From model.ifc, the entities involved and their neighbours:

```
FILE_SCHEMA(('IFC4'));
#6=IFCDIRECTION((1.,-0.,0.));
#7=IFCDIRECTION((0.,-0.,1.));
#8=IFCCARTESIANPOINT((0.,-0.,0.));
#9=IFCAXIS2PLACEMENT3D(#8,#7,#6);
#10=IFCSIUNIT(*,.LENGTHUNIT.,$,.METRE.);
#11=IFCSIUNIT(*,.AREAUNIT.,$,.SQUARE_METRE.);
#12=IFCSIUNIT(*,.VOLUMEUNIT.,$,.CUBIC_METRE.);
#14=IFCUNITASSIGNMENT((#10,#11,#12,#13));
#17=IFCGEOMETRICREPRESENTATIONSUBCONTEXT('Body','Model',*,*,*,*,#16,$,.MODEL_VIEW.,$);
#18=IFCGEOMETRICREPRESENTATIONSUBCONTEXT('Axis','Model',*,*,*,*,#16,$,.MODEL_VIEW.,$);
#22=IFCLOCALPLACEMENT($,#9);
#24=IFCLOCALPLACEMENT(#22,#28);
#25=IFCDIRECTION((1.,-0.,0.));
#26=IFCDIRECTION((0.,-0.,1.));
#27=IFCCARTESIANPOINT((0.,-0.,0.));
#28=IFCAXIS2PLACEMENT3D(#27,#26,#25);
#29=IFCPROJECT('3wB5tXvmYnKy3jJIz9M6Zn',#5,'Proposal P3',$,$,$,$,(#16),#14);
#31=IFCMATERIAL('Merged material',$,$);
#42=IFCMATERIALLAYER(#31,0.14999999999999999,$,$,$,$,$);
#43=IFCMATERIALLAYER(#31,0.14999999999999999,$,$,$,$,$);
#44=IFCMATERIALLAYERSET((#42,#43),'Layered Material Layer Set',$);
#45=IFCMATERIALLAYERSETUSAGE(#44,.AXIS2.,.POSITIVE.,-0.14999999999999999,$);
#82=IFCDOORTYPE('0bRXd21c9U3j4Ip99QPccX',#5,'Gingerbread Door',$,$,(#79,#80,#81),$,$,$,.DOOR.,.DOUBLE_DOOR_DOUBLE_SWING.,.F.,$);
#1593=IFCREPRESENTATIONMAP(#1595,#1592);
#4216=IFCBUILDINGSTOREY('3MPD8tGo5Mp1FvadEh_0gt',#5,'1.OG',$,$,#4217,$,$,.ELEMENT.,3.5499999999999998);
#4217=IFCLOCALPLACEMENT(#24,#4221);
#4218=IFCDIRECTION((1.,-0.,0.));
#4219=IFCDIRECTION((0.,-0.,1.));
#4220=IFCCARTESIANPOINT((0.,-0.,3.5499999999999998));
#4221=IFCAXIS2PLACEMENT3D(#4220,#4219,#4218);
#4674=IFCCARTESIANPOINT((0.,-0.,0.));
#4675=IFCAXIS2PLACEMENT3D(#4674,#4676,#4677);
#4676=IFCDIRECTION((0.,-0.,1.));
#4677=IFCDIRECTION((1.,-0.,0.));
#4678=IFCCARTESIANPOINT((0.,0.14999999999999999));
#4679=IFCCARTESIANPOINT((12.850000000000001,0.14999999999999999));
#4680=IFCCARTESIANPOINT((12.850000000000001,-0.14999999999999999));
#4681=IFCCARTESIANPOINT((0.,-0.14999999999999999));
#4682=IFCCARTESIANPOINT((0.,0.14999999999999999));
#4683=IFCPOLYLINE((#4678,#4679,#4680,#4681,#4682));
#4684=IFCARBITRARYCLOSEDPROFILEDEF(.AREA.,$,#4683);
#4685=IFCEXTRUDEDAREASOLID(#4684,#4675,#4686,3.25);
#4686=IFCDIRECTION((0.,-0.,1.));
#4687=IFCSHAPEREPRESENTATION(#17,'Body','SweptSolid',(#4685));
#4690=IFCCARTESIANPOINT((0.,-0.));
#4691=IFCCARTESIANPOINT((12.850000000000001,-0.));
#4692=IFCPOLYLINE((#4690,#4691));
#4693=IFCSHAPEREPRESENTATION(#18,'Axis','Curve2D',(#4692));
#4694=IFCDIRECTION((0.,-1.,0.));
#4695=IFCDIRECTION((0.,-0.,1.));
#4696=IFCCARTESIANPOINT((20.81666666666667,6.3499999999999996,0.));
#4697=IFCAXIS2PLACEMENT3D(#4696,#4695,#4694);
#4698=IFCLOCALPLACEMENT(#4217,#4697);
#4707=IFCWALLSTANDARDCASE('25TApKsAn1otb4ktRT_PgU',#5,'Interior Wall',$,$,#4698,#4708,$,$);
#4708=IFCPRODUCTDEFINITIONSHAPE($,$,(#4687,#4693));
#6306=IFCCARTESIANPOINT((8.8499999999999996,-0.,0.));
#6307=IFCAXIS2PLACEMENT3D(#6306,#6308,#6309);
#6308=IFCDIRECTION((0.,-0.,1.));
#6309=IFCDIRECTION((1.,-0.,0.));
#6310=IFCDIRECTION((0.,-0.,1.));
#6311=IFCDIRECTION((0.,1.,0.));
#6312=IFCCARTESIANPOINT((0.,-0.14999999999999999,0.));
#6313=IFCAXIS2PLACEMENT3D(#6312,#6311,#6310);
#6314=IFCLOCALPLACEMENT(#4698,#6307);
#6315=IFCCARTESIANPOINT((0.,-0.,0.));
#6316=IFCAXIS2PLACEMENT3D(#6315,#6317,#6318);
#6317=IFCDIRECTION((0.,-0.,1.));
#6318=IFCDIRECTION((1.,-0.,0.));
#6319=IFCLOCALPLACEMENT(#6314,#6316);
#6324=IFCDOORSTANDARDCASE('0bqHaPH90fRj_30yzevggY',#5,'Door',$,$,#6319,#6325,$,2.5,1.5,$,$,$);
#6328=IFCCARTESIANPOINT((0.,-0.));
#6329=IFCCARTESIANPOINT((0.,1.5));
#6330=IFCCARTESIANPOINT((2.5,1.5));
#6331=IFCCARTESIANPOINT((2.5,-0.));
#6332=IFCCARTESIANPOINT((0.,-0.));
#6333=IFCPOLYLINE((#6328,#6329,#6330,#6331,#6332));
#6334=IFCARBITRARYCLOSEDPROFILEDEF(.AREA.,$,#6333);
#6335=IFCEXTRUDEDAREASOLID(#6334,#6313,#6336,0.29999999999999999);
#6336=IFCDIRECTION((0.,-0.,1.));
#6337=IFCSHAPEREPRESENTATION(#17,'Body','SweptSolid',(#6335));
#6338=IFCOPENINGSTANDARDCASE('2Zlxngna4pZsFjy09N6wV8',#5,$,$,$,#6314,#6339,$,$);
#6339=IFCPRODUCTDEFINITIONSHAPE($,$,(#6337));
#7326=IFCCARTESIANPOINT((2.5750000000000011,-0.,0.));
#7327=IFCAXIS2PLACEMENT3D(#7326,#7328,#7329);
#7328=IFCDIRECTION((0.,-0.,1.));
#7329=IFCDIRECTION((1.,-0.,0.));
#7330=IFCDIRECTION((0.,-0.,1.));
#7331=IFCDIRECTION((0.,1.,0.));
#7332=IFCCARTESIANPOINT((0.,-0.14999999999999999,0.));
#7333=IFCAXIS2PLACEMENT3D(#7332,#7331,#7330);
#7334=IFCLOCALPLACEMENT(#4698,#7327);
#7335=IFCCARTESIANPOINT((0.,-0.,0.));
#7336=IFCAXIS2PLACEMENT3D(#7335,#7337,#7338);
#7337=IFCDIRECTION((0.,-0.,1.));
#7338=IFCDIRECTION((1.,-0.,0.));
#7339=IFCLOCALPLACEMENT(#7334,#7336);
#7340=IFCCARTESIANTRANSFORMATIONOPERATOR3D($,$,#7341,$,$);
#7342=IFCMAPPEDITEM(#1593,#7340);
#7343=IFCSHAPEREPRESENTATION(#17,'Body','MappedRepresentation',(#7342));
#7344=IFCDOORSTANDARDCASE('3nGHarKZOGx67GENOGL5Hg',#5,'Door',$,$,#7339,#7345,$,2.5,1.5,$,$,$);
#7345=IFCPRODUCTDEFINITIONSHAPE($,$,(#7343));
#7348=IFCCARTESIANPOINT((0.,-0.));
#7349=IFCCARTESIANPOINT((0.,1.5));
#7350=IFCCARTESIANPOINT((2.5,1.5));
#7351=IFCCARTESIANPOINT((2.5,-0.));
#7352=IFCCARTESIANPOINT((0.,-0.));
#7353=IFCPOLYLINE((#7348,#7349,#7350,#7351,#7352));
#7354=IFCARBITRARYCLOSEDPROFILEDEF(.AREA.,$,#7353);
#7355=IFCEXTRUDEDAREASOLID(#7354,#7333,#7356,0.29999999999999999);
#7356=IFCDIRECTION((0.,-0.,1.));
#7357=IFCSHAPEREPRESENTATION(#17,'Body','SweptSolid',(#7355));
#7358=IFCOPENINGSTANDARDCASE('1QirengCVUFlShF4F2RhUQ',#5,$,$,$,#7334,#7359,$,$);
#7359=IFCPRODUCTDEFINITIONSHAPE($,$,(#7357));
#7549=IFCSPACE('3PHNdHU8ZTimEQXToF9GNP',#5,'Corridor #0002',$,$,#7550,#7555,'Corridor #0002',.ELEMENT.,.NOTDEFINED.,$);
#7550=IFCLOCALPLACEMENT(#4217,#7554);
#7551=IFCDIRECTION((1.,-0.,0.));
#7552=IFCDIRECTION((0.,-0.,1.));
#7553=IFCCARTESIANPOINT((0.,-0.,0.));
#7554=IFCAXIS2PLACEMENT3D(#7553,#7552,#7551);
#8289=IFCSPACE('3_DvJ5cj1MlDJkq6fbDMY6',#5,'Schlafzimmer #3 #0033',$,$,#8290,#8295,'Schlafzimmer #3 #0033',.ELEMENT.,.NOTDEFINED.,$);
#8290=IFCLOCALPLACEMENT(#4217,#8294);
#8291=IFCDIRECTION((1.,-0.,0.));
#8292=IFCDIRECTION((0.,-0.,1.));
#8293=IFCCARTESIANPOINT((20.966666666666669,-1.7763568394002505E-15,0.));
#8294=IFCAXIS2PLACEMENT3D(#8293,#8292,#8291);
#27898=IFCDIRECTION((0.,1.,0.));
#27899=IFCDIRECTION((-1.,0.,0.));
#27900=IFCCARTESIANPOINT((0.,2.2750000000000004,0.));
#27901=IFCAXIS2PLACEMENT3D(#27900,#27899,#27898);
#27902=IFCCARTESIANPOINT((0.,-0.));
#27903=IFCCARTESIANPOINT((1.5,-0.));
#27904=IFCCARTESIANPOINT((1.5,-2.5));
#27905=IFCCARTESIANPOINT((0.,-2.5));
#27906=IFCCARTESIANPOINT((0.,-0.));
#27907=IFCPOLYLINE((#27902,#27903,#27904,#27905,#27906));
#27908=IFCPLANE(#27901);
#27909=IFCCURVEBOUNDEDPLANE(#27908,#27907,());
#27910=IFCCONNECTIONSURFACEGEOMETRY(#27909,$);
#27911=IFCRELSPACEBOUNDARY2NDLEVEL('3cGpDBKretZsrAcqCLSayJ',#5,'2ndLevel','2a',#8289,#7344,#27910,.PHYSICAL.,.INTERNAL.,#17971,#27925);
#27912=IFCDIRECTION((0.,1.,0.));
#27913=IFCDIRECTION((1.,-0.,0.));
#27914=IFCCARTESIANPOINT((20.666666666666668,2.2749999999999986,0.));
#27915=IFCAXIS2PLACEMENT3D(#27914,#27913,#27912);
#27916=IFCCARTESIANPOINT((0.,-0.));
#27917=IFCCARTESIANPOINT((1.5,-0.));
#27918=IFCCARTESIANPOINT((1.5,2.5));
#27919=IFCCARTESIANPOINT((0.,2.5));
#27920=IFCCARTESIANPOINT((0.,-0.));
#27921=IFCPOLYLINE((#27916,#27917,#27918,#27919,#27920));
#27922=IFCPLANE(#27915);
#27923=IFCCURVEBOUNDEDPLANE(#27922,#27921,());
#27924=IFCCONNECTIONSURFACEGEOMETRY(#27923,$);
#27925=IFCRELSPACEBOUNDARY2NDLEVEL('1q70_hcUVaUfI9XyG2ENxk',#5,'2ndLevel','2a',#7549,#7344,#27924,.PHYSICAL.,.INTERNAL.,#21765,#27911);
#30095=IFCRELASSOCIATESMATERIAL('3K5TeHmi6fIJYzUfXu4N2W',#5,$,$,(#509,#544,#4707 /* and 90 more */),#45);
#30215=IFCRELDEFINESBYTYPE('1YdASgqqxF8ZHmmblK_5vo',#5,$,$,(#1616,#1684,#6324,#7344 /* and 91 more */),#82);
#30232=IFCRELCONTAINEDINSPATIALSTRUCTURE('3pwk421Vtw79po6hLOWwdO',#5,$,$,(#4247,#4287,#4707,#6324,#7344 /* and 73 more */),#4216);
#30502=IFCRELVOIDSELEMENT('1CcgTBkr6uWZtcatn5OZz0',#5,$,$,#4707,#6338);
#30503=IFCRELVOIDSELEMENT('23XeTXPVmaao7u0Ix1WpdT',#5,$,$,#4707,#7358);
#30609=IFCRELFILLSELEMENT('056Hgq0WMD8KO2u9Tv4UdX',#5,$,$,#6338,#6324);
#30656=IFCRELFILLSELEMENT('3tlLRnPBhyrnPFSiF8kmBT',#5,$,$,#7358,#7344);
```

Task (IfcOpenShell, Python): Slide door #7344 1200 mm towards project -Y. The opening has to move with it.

```python
import numpy as np
import ifcopenshell
import ifcopenshell.api.geometry
import ifcopenshell.util.placement

model = ifcopenshell.open("model.ifc")

door = model.by_id(7344)
opening = door.FillsVoids[0].RelatingOpeningElement
wall = opening.VoidsElements[0].RelatingBuildingElement

wall_matrix = ifcopenshell.util.placement.get_local_placement(wall.ObjectPlacement)
shift = wall_matrix[:3, 0] * 1.2
before = ifcopenshell.util.placement.get_local_placement(door.ObjectPlacement)[:3, 3].copy()

# The door is placed relative to its opening, so it follows when the opening moves.
matrix = ifcopenshell.util.placement.get_local_placement(opening.ObjectPlacement)
matrix[:3, 3] += shift
ifcopenshell.api.geometry.edit_object_placement(
    model, product=opening, matrix=matrix, is_si=False, should_transform_children=True
)

# Space boundary surfaces are stored in each space's coordinates; move them too.
for rel in door.ProvidesBoundaries:
    if not rel.ConnectionGeometry:
        continue
    surface = rel.ConnectionGeometry.SurfaceOnRelatingElement.BasisSurface
    space_matrix = ifcopenshell.util.placement.get_local_placement(rel.RelatingSpace.ObjectPlacement)
    point = np.array(surface.Position.Location.Coordinates) + space_matrix[:3, :3].T @ shift
    surface.Position = model.createIfcAxis2Placement3D(
        model.createIfcCartesianPoint(point.tolist()), surface.Position.Axis, surface.Position.RefDirection
    )

after = ifcopenshell.util.placement.get_local_placement(door.ObjectPlacement)[:3, 3]
print("door moved by", (after - before).round(3) + 0.0)

model.write("model_edited.ifc")
```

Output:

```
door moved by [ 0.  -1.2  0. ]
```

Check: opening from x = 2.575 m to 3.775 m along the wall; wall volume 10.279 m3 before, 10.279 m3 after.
